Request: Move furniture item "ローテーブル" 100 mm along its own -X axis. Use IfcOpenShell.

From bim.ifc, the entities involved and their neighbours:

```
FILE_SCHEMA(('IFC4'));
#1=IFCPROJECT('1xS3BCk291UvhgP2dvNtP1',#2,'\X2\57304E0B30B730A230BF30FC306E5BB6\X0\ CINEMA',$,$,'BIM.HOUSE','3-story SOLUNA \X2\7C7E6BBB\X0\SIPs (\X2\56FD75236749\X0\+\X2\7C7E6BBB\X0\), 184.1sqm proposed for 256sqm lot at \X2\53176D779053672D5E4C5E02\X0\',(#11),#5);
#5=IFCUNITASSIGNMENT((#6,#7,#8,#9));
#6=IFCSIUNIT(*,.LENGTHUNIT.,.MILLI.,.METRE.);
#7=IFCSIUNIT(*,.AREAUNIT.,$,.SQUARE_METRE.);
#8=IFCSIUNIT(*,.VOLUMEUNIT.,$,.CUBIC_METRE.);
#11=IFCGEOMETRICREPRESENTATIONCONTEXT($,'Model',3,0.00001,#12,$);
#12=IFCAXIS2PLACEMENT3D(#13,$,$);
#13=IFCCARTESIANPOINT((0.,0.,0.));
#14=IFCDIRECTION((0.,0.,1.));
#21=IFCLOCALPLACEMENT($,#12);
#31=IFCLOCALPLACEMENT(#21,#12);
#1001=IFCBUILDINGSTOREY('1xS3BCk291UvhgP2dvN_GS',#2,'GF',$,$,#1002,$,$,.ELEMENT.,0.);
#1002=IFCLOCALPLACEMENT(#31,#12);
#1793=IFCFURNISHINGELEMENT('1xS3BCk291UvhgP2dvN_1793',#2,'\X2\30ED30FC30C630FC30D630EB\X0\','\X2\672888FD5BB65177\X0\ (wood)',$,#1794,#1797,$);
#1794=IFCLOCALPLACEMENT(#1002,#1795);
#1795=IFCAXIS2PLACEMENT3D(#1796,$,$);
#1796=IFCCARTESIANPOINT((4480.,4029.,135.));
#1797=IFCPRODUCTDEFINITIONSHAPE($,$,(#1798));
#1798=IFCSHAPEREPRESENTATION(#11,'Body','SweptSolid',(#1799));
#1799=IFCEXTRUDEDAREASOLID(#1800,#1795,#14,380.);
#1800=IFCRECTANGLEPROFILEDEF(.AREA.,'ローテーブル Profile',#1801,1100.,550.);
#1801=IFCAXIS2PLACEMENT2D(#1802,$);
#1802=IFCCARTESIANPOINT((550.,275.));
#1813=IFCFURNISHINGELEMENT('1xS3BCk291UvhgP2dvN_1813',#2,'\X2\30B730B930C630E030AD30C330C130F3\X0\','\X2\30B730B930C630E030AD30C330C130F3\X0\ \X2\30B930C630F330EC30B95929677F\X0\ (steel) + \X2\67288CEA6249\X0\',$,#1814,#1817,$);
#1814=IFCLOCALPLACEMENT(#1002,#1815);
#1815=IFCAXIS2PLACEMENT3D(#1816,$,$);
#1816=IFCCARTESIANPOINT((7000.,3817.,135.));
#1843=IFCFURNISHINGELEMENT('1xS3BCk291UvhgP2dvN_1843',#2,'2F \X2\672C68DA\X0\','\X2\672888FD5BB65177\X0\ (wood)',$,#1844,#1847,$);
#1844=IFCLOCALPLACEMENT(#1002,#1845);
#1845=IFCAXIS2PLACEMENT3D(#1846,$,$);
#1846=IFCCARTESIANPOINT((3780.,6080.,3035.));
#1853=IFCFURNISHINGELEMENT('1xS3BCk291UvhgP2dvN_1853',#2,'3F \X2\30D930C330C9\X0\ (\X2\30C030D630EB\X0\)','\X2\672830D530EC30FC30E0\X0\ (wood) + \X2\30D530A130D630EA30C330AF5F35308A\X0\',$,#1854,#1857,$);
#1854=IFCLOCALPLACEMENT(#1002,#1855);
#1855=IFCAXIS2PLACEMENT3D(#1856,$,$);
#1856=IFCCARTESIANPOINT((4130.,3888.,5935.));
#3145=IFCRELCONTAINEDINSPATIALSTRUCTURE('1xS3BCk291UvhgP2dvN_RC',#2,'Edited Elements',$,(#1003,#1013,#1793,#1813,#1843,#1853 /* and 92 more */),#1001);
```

```python
import ifcopenshell
import ifcopenshell.api.geometry
import ifcopenshell.util.placement
import ifcopenshell.util.unit

model = ifcopenshell.open("bim.ifc")
unit_scale = ifcopenshell.util.unit.calculate_unit_scale(model)

item = model.by_guid("1xS3BCk291UvhgP2dvN_1793")
matrix = ifcopenshell.util.placement.get_local_placement(item.ObjectPlacement)
matrix[:3, 3] -= matrix[:3, 0] * 0.1 / unit_scale
ifcopenshell.api.geometry.edit_object_placement(model, product=item, matrix=matrix, is_si=False)

print(ifcopenshell.util.placement.get_local_placement(item.ObjectPlacement).round(3) + 0.0)

model.write("bim_v2.ifc")
```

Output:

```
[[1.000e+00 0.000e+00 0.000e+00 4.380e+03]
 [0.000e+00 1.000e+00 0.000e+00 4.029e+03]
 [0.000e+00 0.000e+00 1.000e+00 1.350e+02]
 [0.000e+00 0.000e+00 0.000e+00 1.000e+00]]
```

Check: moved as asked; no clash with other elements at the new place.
